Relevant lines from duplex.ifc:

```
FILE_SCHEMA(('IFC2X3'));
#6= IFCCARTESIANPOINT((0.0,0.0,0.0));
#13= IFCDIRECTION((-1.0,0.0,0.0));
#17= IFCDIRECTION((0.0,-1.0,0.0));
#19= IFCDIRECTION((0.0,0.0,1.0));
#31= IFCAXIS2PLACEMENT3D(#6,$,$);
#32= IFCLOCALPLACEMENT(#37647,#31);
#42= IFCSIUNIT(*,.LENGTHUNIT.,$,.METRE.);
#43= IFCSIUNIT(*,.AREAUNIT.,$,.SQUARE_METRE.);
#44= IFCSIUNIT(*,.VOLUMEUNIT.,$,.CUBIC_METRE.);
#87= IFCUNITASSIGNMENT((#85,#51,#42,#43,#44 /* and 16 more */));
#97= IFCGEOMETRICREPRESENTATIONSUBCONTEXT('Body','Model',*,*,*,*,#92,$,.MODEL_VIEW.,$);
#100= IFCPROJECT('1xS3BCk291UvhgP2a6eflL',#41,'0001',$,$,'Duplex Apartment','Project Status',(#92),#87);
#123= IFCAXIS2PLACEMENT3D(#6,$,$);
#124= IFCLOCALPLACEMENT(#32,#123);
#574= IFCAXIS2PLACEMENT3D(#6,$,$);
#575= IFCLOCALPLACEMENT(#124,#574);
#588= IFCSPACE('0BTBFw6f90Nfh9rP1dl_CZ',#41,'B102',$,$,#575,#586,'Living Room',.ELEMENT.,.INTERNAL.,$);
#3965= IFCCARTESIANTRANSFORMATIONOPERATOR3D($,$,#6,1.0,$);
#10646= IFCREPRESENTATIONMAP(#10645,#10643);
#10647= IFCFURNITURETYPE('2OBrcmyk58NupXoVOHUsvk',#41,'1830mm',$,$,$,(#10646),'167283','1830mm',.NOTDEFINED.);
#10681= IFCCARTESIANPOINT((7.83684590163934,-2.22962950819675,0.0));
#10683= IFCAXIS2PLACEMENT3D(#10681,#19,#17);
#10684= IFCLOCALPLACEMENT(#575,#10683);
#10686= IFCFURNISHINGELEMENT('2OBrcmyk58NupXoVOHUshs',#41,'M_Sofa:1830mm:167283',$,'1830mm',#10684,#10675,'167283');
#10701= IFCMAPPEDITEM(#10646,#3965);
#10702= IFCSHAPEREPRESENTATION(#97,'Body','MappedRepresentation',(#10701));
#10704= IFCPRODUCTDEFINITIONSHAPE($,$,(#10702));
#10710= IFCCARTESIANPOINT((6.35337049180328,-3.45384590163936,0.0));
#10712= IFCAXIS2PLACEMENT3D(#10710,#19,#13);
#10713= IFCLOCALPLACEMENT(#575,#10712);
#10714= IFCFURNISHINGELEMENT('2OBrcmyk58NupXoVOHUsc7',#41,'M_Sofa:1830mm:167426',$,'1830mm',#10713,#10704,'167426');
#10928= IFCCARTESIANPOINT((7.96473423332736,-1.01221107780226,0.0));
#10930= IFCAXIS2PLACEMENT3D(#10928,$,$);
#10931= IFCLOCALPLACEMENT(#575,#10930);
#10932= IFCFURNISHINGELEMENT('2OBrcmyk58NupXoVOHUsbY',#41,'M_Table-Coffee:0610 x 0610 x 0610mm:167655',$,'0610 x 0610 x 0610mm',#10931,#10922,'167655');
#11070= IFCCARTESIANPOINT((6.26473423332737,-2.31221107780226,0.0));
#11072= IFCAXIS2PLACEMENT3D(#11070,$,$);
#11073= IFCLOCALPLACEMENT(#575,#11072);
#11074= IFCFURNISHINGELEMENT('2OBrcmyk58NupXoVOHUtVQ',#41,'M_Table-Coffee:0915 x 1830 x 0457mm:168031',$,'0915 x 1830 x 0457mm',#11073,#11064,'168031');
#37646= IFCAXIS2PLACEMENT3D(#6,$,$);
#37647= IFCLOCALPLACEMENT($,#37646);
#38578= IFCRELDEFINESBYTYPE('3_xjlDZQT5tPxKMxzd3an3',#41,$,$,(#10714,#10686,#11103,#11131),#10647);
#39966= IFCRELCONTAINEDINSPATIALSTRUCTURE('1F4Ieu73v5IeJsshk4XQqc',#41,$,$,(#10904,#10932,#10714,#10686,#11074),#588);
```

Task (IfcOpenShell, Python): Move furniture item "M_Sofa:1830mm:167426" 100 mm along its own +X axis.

```python
import ifcopenshell
import ifcopenshell.api.geometry
import ifcopenshell.util.placement

model = ifcopenshell.open("duplex.ifc")

item = model.by_id(10714)
matrix = ifcopenshell.util.placement.get_local_placement(item.ObjectPlacement)
matrix[:3, 3] += matrix[:3, 0] * 0.1
ifcopenshell.api.geometry.edit_object_placement(model, product=item, matrix=matrix, is_si=False)

print(ifcopenshell.util.placement.get_local_placement(item.ObjectPlacement).round(3) + 0.0)

model.write("duplex-out.ifc")
```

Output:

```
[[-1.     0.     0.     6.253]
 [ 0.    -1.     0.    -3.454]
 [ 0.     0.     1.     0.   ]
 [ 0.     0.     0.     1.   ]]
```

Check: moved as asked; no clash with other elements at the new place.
